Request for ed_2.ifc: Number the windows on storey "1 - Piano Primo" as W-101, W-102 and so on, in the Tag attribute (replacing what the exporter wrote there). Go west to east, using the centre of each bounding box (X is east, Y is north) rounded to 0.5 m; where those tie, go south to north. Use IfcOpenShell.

First a look at what the model holds.

```python
import ifcopenshell
import ifcopenshell.util.element
import ifcopenshell.util.placement

model = ifcopenshell.open("ed_2.ifc")
print(model.schema)
storey = next(s for s in model.by_type("IfcBuildingStorey") if s.Name == "1 - Piano Primo")
windows = [e for e in ifcopenshell.util.element.get_decomposition(storey) if e.is_a("IfcWindow")]
for e in sorted(windows, key=lambda e: e.id()):
    origin = ifcopenshell.util.placement.get_local_placement(e.ObjectPlacement)[:3, 3]
    print(e.id(), e.Tag, e.Name, origin.round(2) + 0.0, sep=" | ")
```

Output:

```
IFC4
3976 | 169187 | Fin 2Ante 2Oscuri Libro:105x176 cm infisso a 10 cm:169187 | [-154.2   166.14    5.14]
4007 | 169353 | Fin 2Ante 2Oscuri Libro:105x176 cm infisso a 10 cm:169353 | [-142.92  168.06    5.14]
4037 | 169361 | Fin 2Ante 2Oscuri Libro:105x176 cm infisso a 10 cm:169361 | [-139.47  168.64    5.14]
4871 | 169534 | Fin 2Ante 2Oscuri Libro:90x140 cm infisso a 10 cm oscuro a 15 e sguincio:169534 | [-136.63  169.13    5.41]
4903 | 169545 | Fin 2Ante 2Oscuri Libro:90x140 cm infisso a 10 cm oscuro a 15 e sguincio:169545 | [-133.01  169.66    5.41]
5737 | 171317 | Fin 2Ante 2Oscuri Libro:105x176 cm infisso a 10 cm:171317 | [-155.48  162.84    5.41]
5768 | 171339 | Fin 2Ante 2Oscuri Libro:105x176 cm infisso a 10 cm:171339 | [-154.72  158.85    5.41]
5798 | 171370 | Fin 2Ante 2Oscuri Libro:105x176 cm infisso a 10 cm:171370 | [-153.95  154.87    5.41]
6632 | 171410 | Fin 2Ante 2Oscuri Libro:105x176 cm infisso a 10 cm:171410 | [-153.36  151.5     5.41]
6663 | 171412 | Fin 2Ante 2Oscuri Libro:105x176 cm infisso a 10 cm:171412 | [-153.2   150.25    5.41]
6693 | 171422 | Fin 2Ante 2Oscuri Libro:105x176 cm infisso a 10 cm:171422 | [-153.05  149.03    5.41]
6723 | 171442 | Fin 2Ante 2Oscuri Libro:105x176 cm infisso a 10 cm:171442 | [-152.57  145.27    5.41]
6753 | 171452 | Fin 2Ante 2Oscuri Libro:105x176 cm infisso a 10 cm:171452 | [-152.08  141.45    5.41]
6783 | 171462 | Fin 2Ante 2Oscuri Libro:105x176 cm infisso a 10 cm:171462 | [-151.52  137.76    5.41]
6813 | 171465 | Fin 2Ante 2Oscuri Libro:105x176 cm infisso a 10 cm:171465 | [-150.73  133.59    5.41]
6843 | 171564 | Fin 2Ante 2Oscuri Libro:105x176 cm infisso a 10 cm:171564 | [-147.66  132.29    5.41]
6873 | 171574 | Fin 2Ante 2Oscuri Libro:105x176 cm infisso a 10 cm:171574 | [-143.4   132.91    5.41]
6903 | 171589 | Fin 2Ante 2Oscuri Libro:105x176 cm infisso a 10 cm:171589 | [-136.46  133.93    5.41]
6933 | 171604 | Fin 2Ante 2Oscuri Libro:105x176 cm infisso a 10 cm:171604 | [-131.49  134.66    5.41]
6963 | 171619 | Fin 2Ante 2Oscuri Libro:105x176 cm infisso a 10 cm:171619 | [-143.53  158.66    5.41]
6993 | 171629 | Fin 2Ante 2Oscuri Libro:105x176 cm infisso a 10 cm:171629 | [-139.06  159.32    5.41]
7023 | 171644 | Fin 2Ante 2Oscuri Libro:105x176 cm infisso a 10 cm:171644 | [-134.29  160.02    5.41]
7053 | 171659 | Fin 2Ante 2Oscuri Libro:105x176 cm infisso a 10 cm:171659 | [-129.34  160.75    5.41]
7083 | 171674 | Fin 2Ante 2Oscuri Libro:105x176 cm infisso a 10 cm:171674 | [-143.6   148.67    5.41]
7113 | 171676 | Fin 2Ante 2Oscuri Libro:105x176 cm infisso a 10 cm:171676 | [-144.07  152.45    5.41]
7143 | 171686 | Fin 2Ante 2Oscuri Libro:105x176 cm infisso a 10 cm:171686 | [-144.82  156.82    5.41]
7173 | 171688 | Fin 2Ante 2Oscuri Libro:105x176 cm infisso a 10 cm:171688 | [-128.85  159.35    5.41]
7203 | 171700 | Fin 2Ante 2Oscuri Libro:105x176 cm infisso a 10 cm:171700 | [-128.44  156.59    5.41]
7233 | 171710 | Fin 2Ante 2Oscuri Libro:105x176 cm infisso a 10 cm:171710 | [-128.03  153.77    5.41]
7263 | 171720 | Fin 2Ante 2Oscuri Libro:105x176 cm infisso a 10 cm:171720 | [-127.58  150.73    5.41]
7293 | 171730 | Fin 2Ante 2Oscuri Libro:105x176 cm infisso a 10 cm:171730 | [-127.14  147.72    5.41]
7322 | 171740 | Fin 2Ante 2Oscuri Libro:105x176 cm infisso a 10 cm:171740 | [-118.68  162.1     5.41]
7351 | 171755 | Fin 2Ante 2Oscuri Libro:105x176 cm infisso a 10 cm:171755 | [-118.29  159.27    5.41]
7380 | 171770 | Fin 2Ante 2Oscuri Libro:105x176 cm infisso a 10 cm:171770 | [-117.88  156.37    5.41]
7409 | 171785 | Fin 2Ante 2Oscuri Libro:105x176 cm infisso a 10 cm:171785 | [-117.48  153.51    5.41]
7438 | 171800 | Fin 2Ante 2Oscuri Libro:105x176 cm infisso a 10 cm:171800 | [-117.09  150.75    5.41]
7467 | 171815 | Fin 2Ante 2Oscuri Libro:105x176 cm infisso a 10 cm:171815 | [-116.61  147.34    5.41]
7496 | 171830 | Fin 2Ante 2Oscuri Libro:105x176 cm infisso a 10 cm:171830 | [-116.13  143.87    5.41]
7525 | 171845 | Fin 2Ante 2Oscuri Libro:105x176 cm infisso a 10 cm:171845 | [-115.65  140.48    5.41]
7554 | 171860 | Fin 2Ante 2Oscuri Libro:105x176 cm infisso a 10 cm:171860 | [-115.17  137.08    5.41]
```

```python
import ifcopenshell
import ifcopenshell.geom
import ifcopenshell.util.element
import ifcopenshell.util.shape

model = ifcopenshell.open("ed_2.ifc")
settings = ifcopenshell.geom.settings()
settings.set("use-world-coords", True)


def centre(element):
    shape = ifcopenshell.geom.create_shape(settings, element)
    return ifcopenshell.util.shape.get_bbox_centroid(shape.geometry)


storey = next(s for s in model.by_type("IfcBuildingStorey") if s.Name == "1 - Piano Primo")
windows = [e for e in ifcopenshell.util.element.get_decomposition(storey) if e.is_a("IfcWindow")]

# Insertion points can sit at a corner or the storey origin, so sort by the geometry (in metres).
centres = {e: centre(e) for e in windows}
windows.sort(key=lambda e: (round(centres[e][0] / 0.5), centres[e][1]))

for i, e in enumerate(windows, start=1):
    number = f"W-1{i:02d}"
    e.Tag = number
    print(e.id(), number)

model.write("ed_2_v2.ifc")
```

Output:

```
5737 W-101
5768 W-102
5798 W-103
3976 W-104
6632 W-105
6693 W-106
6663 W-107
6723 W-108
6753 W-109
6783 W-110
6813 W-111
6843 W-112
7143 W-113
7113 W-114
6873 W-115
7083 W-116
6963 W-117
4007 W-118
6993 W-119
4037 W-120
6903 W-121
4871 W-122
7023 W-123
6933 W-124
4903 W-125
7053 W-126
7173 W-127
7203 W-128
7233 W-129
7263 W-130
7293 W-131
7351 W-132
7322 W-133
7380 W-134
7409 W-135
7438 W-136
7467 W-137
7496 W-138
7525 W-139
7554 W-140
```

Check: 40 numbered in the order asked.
